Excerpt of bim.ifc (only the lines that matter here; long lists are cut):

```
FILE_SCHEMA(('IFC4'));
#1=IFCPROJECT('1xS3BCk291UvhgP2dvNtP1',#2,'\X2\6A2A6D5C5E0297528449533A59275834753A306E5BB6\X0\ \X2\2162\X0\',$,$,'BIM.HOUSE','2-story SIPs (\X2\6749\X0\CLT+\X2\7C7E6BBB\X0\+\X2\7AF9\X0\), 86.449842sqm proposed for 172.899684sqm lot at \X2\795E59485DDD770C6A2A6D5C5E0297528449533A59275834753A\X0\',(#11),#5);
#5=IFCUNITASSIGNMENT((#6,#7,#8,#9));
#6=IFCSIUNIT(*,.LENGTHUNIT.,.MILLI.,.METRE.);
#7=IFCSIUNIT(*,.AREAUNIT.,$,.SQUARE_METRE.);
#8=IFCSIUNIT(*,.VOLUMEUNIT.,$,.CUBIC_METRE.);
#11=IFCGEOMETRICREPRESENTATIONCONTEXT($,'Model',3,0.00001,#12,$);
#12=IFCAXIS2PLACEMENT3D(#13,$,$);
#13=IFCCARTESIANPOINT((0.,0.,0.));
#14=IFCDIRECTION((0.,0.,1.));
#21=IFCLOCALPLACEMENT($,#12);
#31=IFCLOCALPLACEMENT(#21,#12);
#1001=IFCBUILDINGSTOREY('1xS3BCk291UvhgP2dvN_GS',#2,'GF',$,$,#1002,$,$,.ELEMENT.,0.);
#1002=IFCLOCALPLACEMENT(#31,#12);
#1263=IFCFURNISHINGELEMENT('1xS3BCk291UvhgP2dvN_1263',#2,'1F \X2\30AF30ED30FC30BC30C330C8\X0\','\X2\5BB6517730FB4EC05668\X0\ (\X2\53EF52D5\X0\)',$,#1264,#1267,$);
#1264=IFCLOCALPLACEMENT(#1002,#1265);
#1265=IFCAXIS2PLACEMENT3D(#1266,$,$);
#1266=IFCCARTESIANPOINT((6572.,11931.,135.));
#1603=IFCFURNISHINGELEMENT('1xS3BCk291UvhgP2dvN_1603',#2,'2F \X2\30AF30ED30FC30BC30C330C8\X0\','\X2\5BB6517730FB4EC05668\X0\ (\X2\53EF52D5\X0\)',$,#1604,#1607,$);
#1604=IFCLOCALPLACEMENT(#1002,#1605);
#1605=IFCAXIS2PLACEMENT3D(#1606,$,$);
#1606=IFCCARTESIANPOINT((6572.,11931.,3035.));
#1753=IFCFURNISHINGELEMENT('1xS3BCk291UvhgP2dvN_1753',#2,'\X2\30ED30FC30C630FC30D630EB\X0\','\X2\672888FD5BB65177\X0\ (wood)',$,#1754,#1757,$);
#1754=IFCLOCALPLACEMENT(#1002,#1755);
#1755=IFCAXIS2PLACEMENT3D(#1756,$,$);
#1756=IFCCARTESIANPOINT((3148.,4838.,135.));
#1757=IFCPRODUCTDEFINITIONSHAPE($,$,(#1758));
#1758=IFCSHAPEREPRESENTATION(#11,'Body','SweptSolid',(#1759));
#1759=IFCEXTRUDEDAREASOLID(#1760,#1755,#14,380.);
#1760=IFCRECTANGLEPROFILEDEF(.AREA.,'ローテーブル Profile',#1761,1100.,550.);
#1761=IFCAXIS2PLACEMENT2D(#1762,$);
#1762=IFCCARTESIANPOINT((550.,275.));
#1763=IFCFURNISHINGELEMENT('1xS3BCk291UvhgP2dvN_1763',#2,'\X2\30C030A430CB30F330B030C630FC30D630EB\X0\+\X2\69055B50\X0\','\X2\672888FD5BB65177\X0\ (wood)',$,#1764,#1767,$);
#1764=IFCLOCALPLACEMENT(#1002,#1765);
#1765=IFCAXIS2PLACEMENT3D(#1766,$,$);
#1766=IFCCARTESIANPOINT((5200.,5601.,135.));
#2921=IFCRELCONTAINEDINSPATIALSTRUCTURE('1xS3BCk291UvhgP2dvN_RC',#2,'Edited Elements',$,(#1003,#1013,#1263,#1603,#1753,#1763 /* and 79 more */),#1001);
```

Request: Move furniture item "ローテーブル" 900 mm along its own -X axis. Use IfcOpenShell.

```python
import ifcopenshell
import ifcopenshell.api.geometry
import ifcopenshell.util.placement
import ifcopenshell.util.unit

model = ifcopenshell.open("bim.ifc")
unit_scale = ifcopenshell.util.unit.calculate_unit_scale(model)

item = model.by_guid("1xS3BCk291UvhgP2dvN_1753")
matrix = ifcopenshell.util.placement.get_local_placement(item.ObjectPlacement)
matrix[:3, 3] -= matrix[:3, 0] * 0.9 / unit_scale
ifcopenshell.api.geometry.edit_object_placement(model, product=item, matrix=matrix, is_si=False)

print(ifcopenshell.util.placement.get_local_placement(item.ObjectPlacement).round(3) + 0.0)

model.write("bim_rev.ifc")
```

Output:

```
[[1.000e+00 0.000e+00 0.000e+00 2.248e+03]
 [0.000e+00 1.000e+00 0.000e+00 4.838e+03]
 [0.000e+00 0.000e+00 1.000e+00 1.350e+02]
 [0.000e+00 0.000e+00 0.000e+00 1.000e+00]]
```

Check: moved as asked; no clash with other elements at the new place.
